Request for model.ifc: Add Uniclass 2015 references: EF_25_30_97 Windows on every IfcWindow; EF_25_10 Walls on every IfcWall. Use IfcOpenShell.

First a look at what the model holds.

```python
import ifcopenshell

model = ifcopenshell.open("model.ifc")
print(model.schema)
print("classifications:", [c.Name for c in model.by_type("IfcClassification")])
for ifc_class in ("IfcDoor", "IfcRoof", "IfcStair", "IfcWall", "IfcWindow"):
    print(ifc_class, len(model.by_type(ifc_class)))
```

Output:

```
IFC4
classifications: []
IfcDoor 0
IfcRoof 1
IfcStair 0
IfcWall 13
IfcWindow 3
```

```python
import ifcopenshell
import ifcopenshell.api.classification

model = ifcopenshell.open("model.ifc")

system = ifcopenshell.api.classification.add_classification(model, classification="Uniclass 2015")

codes = {
    "IfcWindow": ("EF_25_30_97", "Windows"),
    "IfcWall": ("EF_25_10", "Walls"),
}
for ifc_class, (code, name) in codes.items():
    products = model.by_type(ifc_class)
    ifcopenshell.api.classification.add_reference(
        model, products=products, classification=system, identification=code, name=name
    )
    print(code, len(products))

model.write("model_v2.ifc")
```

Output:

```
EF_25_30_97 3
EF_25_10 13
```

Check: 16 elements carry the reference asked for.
